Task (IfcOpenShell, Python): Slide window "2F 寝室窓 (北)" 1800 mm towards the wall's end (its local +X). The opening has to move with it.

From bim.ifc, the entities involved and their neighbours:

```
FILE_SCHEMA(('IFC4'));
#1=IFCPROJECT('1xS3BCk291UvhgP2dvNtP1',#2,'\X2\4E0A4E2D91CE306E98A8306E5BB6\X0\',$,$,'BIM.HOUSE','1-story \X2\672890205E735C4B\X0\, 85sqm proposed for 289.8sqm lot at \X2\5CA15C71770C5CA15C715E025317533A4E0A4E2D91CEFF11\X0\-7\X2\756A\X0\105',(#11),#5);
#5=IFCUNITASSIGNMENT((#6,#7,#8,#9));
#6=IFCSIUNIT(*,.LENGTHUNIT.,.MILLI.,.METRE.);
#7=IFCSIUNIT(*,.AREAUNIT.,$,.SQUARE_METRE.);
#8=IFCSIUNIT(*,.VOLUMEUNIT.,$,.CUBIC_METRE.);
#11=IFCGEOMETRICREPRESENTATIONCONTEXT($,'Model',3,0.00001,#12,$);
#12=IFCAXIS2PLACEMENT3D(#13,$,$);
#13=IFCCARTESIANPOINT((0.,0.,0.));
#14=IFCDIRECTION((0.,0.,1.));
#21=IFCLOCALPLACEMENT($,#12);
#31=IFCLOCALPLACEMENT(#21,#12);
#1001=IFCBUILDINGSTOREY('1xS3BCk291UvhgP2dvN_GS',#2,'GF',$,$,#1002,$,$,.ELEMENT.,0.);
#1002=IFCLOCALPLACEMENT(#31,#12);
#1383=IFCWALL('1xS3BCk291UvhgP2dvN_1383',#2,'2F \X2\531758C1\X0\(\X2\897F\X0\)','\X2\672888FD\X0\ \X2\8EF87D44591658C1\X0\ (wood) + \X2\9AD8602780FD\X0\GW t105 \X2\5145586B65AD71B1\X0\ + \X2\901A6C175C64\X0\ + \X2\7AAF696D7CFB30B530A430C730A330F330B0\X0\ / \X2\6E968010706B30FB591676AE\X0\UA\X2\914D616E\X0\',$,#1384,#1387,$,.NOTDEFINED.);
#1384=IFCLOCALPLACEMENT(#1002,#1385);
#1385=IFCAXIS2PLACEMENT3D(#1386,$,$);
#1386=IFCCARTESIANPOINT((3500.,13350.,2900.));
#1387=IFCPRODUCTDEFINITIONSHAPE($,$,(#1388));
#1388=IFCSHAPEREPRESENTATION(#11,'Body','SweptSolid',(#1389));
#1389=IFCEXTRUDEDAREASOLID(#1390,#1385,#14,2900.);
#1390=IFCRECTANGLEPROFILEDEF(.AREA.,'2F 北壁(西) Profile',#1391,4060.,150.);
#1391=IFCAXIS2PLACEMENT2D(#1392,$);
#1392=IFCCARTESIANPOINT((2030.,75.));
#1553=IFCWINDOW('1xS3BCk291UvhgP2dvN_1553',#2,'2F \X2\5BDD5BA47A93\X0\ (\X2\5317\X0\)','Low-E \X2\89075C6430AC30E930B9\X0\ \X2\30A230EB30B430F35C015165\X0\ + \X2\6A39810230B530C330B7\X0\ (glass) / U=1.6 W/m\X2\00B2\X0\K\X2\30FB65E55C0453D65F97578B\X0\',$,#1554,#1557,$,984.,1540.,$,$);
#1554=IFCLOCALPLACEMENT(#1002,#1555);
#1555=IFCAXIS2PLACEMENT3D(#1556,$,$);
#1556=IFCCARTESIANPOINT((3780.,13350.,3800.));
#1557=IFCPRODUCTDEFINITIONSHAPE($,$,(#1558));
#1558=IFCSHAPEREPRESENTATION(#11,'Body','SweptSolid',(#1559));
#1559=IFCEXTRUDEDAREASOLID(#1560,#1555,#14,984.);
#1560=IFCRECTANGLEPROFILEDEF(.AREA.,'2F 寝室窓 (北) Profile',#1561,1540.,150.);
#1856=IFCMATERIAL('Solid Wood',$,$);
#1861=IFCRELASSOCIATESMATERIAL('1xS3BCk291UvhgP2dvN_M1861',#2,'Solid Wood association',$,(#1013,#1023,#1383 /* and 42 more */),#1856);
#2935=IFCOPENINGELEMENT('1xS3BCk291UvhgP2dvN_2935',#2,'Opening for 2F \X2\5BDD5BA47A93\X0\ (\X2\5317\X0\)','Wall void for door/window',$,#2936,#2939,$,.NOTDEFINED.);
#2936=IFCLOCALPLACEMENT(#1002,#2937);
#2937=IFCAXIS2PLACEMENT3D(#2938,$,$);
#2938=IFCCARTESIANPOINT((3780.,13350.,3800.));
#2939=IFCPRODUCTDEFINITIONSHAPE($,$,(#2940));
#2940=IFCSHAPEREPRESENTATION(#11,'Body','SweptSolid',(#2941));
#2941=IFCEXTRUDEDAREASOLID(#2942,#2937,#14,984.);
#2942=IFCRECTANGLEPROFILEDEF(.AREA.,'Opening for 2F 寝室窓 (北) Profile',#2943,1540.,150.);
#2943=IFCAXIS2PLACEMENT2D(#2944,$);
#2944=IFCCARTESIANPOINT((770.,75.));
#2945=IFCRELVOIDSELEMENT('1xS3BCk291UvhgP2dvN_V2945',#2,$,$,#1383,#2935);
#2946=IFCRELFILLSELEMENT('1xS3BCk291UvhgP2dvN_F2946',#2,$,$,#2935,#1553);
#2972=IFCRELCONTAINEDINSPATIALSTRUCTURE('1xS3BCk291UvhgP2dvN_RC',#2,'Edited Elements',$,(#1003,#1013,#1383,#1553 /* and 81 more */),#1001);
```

```python
import ifcopenshell
import ifcopenshell.api.geometry
import ifcopenshell.util.placement

model = ifcopenshell.open("bim.ifc")

window = model.by_guid("1xS3BCk291UvhgP2dvN_1553")
opening = window.FillsVoids[0].RelatingOpeningElement
wall = opening.VoidsElements[0].RelatingBuildingElement

wall_matrix = ifcopenshell.util.placement.get_local_placement(wall.ObjectPlacement)
shift = wall_matrix[:3, 0] * 1800.0
before = ifcopenshell.util.placement.get_local_placement(window.ObjectPlacement)[:3, 3].copy()

# The window is not placed relative to its opening, so move both.
for product in (opening, window):
    matrix = ifcopenshell.util.placement.get_local_placement(product.ObjectPlacement)
    matrix[:3, 3] += shift
    ifcopenshell.api.geometry.edit_object_placement(model, product=product, matrix=matrix, is_si=False)

after = ifcopenshell.util.placement.get_local_placement(window.ObjectPlacement)[:3, 3]
print("window moved by", (after - before).round(3) + 0.0)

model.write("bim-out.ifc")
```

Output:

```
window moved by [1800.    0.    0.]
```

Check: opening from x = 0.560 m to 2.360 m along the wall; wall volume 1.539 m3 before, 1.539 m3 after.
